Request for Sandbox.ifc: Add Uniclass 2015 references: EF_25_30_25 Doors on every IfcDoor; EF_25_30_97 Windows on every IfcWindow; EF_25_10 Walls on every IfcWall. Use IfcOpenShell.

First a look at what the model holds.

```python
import ifcopenshell

model = ifcopenshell.open("Sandbox.ifc")
print(model.schema)
print("classifications:", [c.Name for c in model.by_type("IfcClassification")])
for ifc_class in ("IfcDoor", "IfcRoof", "IfcStair", "IfcWall", "IfcWindow"):
    print(ifc_class, len(model.by_type(ifc_class)))
```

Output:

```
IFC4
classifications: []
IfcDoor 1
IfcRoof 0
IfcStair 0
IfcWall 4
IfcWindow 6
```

```python
import ifcopenshell
import ifcopenshell.api.classification

model = ifcopenshell.open("Sandbox.ifc")

system = ifcopenshell.api.classification.add_classification(model, classification="Uniclass 2015")

codes = {
    "IfcDoor": ("EF_25_30_25", "Doors"),
    "IfcWindow": ("EF_25_30_97", "Windows"),
    "IfcWall": ("EF_25_10", "Walls"),
}
for ifc_class, (code, name) in codes.items():
    products = model.by_type(ifc_class)
    ifcopenshell.api.classification.add_reference(
        model, products=products, classification=system, identification=code, name=name
    )
    print(code, len(products))

model.write("Sandbox-out.ifc")
```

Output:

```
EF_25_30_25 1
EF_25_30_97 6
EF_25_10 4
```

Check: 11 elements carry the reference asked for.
